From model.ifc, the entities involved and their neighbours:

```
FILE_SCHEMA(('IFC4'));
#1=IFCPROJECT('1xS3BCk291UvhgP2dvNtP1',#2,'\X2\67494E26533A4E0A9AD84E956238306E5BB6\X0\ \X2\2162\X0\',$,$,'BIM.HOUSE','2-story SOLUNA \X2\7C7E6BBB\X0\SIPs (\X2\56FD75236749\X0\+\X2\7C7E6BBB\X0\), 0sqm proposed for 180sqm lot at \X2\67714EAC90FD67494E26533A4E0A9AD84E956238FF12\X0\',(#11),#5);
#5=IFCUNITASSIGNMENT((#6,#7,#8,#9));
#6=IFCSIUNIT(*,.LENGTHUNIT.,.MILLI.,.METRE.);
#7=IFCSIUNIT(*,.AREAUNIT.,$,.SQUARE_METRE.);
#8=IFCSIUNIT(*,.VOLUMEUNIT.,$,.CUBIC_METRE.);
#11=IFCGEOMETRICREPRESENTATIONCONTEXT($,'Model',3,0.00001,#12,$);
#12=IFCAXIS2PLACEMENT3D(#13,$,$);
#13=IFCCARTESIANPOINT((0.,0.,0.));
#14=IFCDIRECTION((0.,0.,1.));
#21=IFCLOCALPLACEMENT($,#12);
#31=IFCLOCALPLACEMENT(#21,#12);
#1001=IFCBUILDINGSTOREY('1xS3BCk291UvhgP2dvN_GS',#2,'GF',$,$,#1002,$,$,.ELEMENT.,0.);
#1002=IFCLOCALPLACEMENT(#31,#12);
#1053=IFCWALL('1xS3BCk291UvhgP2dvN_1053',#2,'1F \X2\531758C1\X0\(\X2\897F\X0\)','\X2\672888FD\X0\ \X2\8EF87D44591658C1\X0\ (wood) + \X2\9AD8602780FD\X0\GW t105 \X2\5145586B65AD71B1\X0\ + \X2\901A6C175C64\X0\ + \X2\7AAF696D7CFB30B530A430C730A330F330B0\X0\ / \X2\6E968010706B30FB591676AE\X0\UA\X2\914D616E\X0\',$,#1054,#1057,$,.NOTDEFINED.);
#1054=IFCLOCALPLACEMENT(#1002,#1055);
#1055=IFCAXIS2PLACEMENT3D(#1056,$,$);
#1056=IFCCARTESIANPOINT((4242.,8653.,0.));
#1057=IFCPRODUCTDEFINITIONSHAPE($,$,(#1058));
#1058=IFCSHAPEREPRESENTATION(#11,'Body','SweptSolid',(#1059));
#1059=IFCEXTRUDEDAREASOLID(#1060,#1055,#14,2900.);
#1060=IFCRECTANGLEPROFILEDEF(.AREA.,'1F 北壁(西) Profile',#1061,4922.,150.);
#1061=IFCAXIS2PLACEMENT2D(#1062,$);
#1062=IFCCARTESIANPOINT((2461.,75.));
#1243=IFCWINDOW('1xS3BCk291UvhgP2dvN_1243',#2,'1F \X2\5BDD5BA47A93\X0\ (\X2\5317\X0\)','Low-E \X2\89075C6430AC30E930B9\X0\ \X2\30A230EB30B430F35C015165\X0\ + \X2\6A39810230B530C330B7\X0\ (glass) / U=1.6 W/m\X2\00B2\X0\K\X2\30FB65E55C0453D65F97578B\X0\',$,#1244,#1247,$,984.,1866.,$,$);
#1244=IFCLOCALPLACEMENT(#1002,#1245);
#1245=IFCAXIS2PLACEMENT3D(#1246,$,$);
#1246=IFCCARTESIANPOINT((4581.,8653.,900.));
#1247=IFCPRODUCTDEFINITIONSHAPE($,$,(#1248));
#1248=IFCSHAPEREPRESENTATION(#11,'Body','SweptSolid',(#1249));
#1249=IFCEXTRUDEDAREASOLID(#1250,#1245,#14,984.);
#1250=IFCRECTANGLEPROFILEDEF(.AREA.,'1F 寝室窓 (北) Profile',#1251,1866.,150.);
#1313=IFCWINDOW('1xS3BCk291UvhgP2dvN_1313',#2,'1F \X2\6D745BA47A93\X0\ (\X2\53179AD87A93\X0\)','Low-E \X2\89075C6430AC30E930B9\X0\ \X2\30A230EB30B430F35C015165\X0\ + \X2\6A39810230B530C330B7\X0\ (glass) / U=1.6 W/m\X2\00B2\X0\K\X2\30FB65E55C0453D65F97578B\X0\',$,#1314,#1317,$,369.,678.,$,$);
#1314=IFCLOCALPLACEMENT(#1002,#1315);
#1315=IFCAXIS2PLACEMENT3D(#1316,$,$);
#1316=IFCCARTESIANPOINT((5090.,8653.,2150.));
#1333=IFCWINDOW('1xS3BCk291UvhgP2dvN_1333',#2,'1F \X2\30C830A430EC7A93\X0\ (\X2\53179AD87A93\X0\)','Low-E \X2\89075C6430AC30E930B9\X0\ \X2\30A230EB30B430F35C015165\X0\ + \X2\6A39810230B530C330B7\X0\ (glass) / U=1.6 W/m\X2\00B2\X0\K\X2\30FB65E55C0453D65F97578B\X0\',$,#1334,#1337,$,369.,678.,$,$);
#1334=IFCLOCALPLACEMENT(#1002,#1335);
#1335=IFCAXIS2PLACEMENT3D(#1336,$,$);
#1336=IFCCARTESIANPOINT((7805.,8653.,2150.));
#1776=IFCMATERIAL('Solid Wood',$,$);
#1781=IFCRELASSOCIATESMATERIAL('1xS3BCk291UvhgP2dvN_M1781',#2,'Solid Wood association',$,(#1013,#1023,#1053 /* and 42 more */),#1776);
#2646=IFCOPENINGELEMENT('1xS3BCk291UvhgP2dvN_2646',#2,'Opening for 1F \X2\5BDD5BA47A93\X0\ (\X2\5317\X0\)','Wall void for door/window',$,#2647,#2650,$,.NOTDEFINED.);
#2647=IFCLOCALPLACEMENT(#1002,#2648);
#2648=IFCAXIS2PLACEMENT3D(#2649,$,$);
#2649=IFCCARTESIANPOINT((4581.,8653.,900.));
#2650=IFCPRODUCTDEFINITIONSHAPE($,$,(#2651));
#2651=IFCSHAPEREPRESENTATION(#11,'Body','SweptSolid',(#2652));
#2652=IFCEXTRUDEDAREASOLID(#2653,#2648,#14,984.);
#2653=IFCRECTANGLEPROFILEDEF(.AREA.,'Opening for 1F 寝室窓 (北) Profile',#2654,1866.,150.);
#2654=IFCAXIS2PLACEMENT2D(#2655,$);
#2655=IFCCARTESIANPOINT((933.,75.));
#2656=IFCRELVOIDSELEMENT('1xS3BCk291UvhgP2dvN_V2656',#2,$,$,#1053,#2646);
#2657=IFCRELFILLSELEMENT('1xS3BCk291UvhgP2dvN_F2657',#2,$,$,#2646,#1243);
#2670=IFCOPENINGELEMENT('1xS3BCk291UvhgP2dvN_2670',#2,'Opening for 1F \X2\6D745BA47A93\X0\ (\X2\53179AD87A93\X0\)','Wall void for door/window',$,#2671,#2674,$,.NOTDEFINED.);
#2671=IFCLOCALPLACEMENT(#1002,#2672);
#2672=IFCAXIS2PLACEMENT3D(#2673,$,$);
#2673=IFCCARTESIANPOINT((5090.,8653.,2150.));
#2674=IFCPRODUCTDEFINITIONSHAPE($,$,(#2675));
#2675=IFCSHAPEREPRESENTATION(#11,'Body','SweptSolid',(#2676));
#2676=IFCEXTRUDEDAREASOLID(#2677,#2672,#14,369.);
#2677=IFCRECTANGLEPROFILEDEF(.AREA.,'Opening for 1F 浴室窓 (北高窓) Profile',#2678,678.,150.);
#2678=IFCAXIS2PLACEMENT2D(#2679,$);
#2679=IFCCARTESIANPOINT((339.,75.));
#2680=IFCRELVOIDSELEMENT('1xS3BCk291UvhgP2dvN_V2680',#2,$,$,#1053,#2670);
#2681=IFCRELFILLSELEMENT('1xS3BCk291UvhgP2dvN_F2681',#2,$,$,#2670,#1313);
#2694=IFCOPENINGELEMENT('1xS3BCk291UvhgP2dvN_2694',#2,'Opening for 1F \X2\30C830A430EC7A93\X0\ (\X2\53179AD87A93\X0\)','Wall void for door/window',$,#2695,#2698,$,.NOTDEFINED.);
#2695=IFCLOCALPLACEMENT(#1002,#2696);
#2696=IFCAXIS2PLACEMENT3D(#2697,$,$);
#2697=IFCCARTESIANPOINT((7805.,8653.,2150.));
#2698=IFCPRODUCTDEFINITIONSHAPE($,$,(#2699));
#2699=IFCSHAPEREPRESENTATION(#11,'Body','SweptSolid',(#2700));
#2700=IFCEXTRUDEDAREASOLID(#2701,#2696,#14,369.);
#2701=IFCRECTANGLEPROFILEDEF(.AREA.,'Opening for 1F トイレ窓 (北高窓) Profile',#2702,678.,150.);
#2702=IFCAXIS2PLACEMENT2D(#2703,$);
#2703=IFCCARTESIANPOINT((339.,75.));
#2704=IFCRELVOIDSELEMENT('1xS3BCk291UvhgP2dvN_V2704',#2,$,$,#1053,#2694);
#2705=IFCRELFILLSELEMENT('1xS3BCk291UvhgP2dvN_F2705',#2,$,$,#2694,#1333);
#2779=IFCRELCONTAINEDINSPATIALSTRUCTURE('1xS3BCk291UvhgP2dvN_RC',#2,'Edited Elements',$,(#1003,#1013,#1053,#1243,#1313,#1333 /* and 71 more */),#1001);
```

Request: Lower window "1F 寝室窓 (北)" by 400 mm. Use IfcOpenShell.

```python
import numpy as np
import ifcopenshell
import ifcopenshell.api.geometry
import ifcopenshell.util.placement
import ifcopenshell.util.unit

model = ifcopenshell.open("model.ifc")
unit_scale = ifcopenshell.util.unit.calculate_unit_scale(model)

window = model.by_guid("1xS3BCk291UvhgP2dvN_1243")
opening = window.FillsVoids[0].RelatingOpeningElement
dz = -0.4 / unit_scale

shift = np.array([0.0, 0.0, dz])
# The window is not placed relative to its opening, so move both.
for product in (opening, window):
    matrix = ifcopenshell.util.placement.get_local_placement(product.ObjectPlacement)
    matrix[:3, 3] += shift
    ifcopenshell.api.geometry.edit_object_placement(model, product=product, matrix=matrix, is_si=False)

print(f"moved by {dz * unit_scale:+.3f} m")

model.write("model_edited.ifc")
```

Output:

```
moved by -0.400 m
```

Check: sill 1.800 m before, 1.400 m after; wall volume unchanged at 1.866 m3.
